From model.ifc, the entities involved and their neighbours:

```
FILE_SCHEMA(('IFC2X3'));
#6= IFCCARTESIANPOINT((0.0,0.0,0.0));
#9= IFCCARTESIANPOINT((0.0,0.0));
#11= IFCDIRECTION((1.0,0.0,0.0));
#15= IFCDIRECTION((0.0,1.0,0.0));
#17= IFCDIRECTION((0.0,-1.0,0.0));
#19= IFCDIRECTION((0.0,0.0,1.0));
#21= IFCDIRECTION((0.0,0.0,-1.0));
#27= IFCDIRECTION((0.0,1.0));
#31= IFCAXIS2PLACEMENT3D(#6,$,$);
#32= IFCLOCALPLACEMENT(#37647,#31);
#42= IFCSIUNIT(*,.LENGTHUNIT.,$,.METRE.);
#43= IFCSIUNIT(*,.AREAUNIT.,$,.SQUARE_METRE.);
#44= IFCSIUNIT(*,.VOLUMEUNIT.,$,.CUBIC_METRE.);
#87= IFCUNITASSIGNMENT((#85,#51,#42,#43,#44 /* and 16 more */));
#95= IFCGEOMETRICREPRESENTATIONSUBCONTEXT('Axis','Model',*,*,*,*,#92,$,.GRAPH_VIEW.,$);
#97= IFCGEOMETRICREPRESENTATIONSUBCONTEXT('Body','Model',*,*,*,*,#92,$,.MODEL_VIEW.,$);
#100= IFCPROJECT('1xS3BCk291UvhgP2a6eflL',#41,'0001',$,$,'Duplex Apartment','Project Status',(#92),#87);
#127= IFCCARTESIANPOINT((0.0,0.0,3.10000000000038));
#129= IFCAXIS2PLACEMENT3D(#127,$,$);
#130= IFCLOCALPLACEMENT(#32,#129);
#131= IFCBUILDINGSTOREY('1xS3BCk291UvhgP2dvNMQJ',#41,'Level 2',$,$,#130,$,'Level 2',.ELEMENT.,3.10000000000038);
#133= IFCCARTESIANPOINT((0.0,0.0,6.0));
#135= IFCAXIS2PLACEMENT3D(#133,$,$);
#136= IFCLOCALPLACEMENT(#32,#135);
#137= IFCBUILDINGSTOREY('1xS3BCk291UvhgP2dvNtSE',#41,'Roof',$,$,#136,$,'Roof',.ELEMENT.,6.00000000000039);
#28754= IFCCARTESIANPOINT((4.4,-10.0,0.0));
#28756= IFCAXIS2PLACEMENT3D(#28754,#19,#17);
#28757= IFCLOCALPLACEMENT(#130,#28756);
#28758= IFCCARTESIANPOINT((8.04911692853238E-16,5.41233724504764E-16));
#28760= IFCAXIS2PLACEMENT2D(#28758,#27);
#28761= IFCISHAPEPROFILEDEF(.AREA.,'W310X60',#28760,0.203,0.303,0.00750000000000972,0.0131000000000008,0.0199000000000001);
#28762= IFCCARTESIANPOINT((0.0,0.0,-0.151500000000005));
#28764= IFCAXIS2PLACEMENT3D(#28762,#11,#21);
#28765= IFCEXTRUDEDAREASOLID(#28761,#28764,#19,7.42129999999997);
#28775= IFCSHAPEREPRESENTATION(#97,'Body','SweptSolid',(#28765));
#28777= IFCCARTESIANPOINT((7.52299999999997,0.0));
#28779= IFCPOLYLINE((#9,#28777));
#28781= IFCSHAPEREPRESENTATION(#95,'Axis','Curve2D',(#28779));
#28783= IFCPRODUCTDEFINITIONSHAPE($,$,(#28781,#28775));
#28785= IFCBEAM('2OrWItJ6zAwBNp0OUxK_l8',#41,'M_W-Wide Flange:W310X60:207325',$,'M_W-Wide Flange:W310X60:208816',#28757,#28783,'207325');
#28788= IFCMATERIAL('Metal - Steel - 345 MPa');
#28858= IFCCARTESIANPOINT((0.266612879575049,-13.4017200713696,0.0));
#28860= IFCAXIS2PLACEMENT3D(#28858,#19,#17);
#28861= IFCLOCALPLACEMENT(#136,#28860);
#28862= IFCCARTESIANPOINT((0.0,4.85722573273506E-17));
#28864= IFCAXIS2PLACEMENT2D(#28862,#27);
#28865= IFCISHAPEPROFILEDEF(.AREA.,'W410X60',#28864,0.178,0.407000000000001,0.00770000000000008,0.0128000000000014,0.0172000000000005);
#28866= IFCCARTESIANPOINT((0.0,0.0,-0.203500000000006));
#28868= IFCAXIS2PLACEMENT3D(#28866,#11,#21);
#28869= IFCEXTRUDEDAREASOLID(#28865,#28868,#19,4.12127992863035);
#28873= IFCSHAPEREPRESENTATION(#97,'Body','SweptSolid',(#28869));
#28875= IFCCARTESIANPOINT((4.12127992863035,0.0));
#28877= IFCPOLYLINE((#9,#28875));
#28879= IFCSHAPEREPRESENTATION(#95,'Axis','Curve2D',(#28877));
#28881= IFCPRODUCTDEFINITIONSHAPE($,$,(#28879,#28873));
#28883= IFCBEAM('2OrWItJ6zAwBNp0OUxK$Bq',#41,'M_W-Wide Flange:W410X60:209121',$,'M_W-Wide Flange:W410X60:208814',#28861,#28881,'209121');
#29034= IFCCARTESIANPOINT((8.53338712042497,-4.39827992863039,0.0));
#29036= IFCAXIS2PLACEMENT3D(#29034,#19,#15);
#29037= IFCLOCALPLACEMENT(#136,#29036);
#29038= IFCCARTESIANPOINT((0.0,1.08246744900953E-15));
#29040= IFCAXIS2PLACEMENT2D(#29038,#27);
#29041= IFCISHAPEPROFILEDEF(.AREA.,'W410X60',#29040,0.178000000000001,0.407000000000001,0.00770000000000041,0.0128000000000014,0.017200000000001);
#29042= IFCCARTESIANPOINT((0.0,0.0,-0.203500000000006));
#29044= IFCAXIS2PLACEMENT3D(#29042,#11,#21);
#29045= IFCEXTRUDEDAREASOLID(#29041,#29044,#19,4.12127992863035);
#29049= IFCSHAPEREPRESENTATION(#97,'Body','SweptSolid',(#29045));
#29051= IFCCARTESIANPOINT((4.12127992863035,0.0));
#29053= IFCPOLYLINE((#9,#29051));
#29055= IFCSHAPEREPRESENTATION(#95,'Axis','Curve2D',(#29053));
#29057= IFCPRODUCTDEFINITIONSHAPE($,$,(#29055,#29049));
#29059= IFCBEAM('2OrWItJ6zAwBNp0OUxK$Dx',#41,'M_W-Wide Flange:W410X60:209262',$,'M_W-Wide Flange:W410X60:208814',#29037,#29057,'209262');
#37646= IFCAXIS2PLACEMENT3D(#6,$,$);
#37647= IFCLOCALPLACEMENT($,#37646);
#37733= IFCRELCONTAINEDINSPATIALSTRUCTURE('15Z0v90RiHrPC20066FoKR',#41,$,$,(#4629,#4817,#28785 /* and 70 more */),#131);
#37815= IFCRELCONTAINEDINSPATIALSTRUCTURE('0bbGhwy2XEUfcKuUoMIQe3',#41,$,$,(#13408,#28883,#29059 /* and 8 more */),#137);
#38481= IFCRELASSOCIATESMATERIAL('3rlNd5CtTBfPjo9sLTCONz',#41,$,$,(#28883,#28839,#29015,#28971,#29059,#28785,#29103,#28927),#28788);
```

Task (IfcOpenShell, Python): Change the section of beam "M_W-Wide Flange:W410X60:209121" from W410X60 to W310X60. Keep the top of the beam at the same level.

```python
import ifcopenshell
import ifcopenshell.util.element
import ifcopenshell.util.representation

model = ifcopenshell.open("model.ifc")

member = model.by_guid("2OrWItJ6zAwBNp0OUxK$Bq")
source = next(p for p in model.by_type("IfcIShapeProfileDef") if p.ProfileName == "W310X60")

body = ifcopenshell.util.representation.get_representation(member, "Model", "Body")
solid = body.Items[0]
old_profile = solid.SweptArea

# Copy the section's sizes but keep this member's own profile position.
profile = ifcopenshell.util.element.copy(model, source)
# Profiles are centred, so shift by half the change in depth to hold the top.
shift = (old_profile.OverallDepth - profile.OverallDepth) / 2
x, y = old_profile.Position.Location.Coordinates
up = (-1.0, 0.0)  # upwards, in the solid's own plane
location = model.createIfcCartesianPoint((x + up[0] * shift, y + up[1] * shift))
profile.Position = model.createIfcAxis2Placement2D(location, old_profile.Position.RefDirection)
solid.SweptArea = profile
if not model.get_total_inverses(old_profile):
    ifcopenshell.util.element.remove_deep2(model, old_profile)
member.Name = member.Name.replace("W410X60", "W310X60")
member.ObjectType = member.ObjectType.replace("W410X60", "W310X60")

print(solid.SweptArea)

model.write("model_rev.ifc")
```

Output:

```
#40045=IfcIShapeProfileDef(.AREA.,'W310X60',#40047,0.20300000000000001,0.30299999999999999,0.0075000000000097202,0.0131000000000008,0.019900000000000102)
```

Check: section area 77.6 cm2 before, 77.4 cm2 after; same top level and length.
